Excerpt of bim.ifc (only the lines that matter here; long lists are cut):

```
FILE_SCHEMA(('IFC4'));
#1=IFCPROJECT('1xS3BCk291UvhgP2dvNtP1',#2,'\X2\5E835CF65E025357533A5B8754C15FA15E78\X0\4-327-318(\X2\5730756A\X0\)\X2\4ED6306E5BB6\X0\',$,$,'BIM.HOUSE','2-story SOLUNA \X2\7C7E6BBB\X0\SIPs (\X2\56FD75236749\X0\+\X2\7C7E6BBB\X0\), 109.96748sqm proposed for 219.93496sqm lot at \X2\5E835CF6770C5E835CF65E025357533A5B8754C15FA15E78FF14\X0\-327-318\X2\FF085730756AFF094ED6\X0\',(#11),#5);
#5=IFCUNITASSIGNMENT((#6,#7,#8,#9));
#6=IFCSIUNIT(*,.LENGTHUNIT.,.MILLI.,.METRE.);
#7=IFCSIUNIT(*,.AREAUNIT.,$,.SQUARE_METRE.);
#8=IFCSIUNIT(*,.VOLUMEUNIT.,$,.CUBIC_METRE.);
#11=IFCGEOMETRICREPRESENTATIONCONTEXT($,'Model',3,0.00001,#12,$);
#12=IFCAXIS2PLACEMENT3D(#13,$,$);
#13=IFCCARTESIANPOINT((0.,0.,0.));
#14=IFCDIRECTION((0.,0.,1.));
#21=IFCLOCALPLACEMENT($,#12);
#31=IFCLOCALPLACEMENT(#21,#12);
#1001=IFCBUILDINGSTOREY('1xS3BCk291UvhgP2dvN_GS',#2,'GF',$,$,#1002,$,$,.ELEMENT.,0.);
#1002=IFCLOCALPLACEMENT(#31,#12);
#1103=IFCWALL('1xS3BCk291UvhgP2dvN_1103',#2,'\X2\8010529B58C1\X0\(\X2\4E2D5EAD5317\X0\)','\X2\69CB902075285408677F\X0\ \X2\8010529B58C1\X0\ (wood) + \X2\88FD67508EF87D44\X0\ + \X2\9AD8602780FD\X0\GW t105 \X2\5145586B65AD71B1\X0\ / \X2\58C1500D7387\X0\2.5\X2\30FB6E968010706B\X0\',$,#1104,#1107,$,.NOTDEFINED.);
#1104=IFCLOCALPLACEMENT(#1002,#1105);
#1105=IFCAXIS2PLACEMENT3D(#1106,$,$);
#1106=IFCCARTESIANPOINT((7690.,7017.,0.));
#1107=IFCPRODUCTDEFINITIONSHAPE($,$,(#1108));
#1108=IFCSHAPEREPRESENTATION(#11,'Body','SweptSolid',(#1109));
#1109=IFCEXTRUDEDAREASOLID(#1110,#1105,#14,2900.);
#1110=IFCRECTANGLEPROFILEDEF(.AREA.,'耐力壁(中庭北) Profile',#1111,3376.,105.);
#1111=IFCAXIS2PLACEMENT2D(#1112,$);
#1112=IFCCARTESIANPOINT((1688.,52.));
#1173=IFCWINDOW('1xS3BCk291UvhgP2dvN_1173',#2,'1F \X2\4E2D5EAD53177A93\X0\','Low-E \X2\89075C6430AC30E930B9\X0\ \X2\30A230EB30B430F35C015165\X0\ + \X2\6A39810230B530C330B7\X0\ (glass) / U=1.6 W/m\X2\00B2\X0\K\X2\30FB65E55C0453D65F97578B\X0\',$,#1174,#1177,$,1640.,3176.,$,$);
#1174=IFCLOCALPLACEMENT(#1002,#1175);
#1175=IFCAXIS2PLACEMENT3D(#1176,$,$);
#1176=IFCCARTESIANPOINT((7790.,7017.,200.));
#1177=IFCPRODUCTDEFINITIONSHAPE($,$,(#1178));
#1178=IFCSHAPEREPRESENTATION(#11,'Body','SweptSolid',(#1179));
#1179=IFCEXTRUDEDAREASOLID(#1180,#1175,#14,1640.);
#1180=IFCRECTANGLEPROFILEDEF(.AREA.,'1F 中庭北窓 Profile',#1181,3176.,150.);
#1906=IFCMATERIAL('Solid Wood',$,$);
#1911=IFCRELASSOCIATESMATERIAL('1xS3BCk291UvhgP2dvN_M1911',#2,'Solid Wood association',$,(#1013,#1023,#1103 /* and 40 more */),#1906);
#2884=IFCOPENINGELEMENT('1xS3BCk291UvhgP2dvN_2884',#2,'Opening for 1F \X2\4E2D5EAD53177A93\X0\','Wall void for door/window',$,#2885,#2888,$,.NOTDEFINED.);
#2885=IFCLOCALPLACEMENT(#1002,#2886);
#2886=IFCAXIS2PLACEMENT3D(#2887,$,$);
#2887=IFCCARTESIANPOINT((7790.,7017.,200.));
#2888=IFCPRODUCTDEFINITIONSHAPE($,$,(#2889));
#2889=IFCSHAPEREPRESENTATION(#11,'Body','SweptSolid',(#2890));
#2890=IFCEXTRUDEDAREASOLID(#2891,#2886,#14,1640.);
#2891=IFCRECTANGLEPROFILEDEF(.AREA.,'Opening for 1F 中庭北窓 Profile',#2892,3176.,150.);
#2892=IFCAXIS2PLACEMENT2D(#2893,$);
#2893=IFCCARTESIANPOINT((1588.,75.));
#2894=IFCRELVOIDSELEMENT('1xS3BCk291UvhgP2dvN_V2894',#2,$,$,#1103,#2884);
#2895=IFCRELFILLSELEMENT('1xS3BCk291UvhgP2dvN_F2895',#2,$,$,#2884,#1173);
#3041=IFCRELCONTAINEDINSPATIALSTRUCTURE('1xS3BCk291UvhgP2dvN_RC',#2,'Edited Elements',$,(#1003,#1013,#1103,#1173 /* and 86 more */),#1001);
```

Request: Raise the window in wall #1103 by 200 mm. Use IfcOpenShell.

```python
import numpy as np
import ifcopenshell
import ifcopenshell.api.geometry
import ifcopenshell.util.placement
import ifcopenshell.util.unit

model = ifcopenshell.open("bim.ifc")
unit_scale = ifcopenshell.util.unit.calculate_unit_scale(model)

window = model.by_guid("1xS3BCk291UvhgP2dvN_1173")
opening = window.FillsVoids[0].RelatingOpeningElement
dz = 0.2 / unit_scale

shift = np.array([0.0, 0.0, dz])
# The window is not placed relative to its opening, so move both.
for product in (opening, window):
    matrix = ifcopenshell.util.placement.get_local_placement(product.ObjectPlacement)
    matrix[:3, 3] += shift
    ifcopenshell.api.geometry.edit_object_placement(model, product=product, matrix=matrix, is_si=False)

print(f"moved by {dz * unit_scale:+.3f} m")

model.write("bim_v2.ifc")
```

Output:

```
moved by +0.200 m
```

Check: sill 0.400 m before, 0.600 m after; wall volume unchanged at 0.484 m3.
